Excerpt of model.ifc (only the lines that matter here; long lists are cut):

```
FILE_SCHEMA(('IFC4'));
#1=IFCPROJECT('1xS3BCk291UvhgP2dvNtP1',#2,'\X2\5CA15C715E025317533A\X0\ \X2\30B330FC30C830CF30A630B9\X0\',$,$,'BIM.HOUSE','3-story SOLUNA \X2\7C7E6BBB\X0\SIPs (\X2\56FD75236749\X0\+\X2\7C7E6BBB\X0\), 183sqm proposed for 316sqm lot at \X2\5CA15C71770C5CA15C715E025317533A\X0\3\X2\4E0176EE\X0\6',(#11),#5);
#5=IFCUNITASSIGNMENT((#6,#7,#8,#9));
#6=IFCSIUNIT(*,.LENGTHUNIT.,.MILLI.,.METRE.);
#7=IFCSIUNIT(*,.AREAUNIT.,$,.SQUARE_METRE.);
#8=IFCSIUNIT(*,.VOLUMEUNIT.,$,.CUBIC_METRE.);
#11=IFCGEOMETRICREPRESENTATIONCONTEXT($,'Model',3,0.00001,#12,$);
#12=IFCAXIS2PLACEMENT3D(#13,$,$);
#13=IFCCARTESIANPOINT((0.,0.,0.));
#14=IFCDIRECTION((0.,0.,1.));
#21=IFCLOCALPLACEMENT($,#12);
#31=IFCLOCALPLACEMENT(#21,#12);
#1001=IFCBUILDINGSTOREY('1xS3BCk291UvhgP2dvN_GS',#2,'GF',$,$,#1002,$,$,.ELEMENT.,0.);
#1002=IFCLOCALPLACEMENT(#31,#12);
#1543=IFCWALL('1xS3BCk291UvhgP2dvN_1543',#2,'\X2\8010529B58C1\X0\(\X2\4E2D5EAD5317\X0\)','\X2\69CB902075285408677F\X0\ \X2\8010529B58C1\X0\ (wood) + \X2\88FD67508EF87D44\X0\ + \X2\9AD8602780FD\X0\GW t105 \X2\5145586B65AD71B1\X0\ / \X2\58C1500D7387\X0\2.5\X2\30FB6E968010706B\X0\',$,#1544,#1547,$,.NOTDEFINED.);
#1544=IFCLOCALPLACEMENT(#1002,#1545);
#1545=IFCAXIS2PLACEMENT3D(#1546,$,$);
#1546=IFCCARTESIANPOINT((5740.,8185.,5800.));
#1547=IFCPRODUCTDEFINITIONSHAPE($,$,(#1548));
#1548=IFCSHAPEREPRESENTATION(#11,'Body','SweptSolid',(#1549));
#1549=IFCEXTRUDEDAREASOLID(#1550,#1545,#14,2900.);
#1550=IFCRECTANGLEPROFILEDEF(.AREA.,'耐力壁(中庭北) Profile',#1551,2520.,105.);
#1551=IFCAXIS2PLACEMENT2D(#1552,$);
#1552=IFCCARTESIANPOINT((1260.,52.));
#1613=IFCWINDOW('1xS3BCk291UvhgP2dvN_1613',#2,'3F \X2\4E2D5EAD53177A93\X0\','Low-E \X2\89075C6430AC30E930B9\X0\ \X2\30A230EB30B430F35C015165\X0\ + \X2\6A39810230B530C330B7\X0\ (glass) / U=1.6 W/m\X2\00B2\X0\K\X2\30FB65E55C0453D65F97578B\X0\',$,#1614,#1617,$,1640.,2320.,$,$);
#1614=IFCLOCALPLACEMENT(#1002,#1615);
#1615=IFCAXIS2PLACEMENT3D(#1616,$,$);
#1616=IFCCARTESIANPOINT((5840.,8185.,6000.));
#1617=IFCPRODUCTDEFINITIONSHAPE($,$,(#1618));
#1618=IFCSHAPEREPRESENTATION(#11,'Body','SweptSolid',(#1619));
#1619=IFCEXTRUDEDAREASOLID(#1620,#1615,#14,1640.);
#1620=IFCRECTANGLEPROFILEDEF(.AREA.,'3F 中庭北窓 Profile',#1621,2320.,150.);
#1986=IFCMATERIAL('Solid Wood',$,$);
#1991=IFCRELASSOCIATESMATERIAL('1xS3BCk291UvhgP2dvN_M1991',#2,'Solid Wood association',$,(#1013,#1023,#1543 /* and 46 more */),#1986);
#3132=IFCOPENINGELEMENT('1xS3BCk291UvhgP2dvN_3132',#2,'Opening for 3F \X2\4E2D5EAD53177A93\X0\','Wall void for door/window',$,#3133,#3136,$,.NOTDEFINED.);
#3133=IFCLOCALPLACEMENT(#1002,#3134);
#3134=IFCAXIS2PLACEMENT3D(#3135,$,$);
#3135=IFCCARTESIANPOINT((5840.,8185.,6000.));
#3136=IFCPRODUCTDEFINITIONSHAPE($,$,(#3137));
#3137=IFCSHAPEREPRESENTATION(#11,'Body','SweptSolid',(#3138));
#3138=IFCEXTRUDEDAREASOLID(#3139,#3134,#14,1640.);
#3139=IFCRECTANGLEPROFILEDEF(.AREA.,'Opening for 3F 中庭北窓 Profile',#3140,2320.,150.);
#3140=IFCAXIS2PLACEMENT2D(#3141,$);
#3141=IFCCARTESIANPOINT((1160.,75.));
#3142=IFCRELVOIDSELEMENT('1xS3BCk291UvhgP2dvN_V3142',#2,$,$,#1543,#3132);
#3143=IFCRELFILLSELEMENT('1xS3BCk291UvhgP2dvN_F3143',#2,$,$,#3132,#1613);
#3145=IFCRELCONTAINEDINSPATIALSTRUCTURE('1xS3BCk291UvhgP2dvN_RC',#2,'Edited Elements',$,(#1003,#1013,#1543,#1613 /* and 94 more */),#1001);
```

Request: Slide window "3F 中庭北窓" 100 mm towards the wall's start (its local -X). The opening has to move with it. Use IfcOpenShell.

```python
import ifcopenshell
import ifcopenshell.api.geometry
import ifcopenshell.util.placement
import ifcopenshell.util.unit

model = ifcopenshell.open("model.ifc")
unit_scale = ifcopenshell.util.unit.calculate_unit_scale(model)

window = model.by_id(1613)
opening = window.FillsVoids[0].RelatingOpeningElement
wall = opening.VoidsElements[0].RelatingBuildingElement

wall_matrix = ifcopenshell.util.placement.get_local_placement(wall.ObjectPlacement)
shift = wall_matrix[:3, 0] * -0.1 / unit_scale
before = ifcopenshell.util.placement.get_local_placement(window.ObjectPlacement)[:3, 3].copy()

# The window is not placed relative to its opening, so move both.
for product in (opening, window):
    matrix = ifcopenshell.util.placement.get_local_placement(product.ObjectPlacement)
    matrix[:3, 3] += shift
    ifcopenshell.api.geometry.edit_object_placement(model, product=product, matrix=matrix, is_si=False)

after = ifcopenshell.util.placement.get_local_placement(window.ObjectPlacement)[:3, 3]
print("window moved by", (after - before).round(3) + 0.0)

model.write("model_edited.ifc")
```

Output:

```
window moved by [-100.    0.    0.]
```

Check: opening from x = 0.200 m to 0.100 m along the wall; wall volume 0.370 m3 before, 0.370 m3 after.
